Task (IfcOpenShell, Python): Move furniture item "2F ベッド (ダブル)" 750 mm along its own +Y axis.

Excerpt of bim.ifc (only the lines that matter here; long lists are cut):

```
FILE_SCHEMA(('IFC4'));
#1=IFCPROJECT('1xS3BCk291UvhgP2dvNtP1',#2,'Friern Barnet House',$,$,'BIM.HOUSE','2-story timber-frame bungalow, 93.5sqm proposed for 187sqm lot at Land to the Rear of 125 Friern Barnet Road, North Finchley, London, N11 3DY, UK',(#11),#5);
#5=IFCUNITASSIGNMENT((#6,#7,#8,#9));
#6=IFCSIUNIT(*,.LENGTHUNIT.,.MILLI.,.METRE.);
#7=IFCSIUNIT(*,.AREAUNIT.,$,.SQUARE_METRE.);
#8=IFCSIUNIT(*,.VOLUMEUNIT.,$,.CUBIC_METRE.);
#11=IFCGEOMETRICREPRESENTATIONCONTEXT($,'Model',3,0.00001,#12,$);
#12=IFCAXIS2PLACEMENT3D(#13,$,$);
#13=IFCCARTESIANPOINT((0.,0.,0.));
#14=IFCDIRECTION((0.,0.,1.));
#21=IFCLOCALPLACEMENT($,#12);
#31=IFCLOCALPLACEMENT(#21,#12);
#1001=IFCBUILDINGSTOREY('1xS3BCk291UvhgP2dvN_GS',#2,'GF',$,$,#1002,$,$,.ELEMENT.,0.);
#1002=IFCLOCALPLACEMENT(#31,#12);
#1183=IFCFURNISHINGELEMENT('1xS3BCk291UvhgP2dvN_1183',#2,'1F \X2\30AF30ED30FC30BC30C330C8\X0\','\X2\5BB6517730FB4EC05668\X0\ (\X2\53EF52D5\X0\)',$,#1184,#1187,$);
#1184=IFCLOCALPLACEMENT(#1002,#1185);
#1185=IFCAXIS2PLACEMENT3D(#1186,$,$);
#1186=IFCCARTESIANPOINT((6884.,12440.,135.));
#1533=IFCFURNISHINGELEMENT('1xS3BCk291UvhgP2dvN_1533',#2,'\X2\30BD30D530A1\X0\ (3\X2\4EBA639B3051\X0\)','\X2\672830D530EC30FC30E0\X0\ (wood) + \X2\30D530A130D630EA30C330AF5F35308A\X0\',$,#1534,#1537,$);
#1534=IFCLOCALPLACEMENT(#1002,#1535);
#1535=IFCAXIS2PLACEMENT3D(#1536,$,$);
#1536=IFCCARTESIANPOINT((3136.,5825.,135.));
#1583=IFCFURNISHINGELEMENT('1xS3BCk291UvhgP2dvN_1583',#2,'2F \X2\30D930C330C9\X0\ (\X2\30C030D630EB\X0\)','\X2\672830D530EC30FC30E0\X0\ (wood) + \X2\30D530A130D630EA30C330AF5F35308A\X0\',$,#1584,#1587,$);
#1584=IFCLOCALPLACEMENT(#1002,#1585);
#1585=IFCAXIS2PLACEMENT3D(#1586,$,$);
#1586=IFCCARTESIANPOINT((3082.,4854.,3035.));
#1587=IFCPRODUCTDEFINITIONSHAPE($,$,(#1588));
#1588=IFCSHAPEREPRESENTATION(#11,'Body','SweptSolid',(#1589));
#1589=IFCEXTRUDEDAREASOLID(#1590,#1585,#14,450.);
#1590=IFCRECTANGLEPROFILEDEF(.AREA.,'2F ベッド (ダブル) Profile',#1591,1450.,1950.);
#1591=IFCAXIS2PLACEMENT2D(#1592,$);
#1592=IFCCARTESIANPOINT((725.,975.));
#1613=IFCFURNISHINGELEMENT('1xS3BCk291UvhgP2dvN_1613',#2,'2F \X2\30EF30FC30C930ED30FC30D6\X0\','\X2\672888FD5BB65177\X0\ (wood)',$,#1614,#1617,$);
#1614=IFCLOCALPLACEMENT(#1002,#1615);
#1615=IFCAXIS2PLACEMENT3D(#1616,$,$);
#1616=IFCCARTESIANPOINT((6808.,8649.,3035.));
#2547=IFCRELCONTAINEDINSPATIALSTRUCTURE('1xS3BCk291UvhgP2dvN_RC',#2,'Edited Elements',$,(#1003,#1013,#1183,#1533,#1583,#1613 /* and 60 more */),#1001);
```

```python
import ifcopenshell
import ifcopenshell.api.geometry
import ifcopenshell.util.placement
import ifcopenshell.util.unit

model = ifcopenshell.open("bim.ifc")
unit_scale = ifcopenshell.util.unit.calculate_unit_scale(model)

item = model.by_id(1583)
matrix = ifcopenshell.util.placement.get_local_placement(item.ObjectPlacement)
matrix[:3, 3] += matrix[:3, 1] * 0.75 / unit_scale
ifcopenshell.api.geometry.edit_object_placement(model, product=item, matrix=matrix, is_si=False)

print(ifcopenshell.util.placement.get_local_placement(item.ObjectPlacement).round(3) + 0.0)

model.write("bim_v2.ifc")
```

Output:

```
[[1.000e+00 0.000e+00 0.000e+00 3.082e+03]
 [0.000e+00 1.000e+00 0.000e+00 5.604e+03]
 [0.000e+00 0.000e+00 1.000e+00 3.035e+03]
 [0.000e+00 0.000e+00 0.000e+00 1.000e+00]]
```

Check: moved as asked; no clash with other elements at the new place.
